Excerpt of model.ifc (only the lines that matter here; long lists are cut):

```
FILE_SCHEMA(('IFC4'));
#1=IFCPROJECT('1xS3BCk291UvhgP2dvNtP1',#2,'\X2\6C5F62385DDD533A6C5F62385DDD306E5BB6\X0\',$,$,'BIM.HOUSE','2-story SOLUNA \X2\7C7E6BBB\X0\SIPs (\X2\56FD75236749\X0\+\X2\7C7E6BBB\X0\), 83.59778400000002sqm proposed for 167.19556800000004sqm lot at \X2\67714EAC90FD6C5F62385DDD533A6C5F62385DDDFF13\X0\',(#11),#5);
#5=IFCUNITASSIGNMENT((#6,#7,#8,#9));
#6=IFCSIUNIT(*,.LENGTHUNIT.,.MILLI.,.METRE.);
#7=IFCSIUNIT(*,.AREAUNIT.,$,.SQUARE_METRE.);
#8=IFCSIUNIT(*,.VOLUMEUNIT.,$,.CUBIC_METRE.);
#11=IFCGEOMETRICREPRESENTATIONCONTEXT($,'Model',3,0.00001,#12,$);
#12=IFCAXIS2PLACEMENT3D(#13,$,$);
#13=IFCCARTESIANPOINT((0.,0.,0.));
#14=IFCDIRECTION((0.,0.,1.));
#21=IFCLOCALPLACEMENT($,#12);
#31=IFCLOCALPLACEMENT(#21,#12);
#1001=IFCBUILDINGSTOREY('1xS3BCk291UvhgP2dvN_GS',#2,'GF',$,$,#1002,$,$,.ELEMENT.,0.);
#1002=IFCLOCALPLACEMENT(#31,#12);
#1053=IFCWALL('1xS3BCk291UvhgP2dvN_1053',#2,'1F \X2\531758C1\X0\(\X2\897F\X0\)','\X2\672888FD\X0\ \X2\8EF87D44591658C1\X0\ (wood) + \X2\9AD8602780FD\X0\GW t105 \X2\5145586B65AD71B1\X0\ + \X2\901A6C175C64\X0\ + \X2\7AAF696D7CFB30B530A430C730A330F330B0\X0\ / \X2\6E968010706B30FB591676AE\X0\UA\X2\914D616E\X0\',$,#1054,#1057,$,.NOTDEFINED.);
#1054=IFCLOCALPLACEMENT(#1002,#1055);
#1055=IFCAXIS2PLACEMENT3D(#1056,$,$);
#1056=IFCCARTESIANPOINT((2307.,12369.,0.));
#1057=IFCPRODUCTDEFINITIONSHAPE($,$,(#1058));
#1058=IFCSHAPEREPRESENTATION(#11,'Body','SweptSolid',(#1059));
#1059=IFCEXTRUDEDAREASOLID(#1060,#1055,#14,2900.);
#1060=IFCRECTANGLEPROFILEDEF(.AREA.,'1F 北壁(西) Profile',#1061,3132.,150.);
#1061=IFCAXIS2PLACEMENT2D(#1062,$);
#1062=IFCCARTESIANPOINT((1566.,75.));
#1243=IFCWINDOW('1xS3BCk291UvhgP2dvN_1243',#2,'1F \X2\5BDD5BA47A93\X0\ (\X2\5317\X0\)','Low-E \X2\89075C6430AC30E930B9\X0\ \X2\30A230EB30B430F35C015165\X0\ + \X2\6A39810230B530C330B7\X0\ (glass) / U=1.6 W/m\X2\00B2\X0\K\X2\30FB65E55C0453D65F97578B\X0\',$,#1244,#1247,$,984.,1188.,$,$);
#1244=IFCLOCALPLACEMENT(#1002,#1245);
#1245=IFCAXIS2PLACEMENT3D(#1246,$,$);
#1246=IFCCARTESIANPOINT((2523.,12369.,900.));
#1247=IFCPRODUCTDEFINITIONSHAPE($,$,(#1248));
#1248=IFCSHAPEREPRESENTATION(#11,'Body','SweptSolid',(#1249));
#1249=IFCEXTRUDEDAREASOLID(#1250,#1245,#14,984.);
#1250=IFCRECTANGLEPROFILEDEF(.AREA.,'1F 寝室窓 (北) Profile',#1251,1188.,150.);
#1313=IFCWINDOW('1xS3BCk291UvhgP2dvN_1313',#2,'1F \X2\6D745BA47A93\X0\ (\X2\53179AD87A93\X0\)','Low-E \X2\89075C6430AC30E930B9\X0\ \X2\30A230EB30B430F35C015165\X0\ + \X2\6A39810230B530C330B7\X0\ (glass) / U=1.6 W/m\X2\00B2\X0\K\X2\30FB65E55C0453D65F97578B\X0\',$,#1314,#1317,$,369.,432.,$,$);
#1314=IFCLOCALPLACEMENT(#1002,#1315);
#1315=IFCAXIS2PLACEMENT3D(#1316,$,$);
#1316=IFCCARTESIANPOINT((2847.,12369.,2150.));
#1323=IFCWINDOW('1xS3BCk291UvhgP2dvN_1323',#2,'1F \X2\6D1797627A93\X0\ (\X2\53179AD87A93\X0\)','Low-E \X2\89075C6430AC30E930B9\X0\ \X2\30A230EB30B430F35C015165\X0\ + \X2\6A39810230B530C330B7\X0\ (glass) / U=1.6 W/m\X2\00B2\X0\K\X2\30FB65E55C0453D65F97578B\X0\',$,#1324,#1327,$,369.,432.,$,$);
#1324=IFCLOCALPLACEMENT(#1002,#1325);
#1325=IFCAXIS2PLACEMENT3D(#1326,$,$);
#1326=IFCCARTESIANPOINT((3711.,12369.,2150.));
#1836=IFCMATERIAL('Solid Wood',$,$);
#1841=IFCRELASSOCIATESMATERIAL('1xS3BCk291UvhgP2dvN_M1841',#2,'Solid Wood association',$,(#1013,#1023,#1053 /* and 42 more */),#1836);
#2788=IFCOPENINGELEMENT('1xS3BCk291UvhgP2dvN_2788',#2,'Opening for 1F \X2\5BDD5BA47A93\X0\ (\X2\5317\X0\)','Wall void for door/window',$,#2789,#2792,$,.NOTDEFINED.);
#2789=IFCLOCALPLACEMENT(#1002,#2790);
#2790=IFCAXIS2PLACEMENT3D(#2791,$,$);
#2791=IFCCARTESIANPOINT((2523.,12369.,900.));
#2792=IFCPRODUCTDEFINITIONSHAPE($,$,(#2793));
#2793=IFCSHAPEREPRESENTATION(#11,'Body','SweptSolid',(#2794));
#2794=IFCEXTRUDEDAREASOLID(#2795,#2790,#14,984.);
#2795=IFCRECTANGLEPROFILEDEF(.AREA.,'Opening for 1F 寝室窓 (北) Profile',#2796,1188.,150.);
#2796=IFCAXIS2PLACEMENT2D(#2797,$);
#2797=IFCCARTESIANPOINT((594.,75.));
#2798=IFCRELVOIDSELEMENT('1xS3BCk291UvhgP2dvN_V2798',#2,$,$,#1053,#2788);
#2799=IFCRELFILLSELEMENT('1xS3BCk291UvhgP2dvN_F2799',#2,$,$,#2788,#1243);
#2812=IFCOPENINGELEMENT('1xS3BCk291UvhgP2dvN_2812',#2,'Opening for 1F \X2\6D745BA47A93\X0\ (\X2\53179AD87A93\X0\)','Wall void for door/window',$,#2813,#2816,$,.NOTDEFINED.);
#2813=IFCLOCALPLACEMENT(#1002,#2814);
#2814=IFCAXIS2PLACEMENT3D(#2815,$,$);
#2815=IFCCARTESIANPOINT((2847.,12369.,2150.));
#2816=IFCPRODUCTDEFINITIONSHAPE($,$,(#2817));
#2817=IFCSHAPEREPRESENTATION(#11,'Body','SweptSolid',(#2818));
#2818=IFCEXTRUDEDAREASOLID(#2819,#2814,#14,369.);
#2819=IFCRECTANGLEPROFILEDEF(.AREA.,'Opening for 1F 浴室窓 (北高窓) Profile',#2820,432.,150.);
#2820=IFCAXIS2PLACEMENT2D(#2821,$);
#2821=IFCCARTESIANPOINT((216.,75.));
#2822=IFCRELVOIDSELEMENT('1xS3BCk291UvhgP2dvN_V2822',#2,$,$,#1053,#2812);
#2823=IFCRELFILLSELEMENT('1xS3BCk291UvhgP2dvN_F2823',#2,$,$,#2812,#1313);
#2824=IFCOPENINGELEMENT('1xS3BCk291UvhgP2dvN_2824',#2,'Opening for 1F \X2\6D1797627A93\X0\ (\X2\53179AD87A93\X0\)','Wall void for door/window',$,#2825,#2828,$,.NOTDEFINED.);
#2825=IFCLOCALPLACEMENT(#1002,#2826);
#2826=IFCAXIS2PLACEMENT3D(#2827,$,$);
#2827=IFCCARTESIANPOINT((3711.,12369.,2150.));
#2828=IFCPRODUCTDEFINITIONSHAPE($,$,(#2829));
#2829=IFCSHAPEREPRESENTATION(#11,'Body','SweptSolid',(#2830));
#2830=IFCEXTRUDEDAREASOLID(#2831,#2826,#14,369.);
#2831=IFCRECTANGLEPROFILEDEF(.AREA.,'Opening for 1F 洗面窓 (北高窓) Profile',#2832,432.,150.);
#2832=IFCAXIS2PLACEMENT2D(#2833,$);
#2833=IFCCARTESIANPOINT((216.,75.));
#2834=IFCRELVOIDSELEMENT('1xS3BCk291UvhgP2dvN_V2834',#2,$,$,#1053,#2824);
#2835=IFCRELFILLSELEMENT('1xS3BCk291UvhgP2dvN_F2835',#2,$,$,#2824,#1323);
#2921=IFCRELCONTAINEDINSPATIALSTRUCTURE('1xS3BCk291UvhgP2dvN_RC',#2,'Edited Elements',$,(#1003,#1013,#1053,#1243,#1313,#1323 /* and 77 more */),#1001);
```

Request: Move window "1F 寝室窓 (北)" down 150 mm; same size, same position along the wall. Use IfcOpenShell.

```python
import numpy as np
import ifcopenshell
import ifcopenshell.api.geometry
import ifcopenshell.util.placement
import ifcopenshell.util.unit

model = ifcopenshell.open("model.ifc")
unit_scale = ifcopenshell.util.unit.calculate_unit_scale(model)

window = model.by_id(1243)
opening = window.FillsVoids[0].RelatingOpeningElement
dz = -0.15 / unit_scale

shift = np.array([0.0, 0.0, dz])
# The window is not placed relative to its opening, so move both.
for product in (opening, window):
    matrix = ifcopenshell.util.placement.get_local_placement(product.ObjectPlacement)
    matrix[:3, 3] += shift
    ifcopenshell.api.geometry.edit_object_placement(model, product=product, matrix=matrix, is_si=False)

print(f"moved by {dz * unit_scale:+.3f} m")

model.write("model_v2.ifc")
```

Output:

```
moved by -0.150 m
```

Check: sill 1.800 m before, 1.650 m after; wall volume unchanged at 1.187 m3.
